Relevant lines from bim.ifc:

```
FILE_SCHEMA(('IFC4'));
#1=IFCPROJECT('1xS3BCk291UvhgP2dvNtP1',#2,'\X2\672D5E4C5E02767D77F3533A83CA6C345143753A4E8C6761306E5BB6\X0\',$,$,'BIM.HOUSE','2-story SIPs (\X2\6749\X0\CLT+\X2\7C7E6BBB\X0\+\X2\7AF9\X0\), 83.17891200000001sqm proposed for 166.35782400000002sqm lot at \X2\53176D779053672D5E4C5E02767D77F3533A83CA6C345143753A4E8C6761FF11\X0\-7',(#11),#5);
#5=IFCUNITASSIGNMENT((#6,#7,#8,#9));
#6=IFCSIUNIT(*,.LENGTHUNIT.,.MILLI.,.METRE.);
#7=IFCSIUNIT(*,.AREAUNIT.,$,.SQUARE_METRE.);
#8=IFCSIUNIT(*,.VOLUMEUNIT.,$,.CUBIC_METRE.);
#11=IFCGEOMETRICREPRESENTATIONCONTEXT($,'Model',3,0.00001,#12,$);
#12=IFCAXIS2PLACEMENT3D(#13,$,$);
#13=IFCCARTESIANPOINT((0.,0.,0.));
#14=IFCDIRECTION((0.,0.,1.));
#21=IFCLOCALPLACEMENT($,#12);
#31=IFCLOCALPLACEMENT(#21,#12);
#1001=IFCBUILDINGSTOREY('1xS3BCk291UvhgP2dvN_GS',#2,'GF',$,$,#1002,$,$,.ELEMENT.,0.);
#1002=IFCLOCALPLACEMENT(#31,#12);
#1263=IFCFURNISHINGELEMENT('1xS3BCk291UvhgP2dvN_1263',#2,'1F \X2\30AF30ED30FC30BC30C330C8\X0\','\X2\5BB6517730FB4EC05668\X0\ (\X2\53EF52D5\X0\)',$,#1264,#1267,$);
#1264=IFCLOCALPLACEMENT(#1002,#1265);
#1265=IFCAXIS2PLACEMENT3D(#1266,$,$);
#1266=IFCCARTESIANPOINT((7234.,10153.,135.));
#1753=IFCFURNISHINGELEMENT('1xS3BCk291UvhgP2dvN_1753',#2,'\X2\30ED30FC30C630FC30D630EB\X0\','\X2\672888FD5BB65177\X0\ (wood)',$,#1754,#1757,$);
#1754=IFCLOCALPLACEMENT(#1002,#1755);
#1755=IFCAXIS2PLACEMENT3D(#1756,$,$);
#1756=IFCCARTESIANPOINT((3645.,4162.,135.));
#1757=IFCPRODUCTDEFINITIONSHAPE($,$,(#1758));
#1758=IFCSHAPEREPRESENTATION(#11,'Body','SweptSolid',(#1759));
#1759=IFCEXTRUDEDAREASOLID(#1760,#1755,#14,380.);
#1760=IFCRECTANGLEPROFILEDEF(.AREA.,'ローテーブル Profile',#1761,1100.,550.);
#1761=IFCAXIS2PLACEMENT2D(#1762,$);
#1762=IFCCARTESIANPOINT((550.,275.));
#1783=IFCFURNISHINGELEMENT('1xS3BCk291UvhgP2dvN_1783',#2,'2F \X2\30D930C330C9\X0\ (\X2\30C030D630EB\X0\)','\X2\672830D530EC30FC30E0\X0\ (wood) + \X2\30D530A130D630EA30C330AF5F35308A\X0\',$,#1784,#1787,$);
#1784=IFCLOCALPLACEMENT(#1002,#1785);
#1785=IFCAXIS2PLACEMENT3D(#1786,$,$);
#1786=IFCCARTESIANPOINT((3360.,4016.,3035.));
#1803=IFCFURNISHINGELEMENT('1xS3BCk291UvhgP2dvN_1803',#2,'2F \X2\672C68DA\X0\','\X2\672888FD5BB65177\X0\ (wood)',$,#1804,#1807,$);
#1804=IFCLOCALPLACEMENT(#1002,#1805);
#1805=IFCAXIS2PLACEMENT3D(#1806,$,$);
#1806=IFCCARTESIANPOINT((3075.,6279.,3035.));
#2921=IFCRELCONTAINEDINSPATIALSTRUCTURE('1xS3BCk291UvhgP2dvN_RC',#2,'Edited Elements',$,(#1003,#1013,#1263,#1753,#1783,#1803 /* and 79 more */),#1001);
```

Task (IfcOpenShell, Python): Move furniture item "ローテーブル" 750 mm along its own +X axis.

```python
import ifcopenshell
import ifcopenshell.api.geometry
import ifcopenshell.util.placement
import ifcopenshell.util.unit

model = ifcopenshell.open("bim.ifc")
unit_scale = ifcopenshell.util.unit.calculate_unit_scale(model)

item = model.by_id(1753)
matrix = ifcopenshell.util.placement.get_local_placement(item.ObjectPlacement)
matrix[:3, 3] += matrix[:3, 0] * 0.75 / unit_scale
ifcopenshell.api.geometry.edit_object_placement(model, product=item, matrix=matrix, is_si=False)

print(ifcopenshell.util.placement.get_local_placement(item.ObjectPlacement).round(3) + 0.0)

model.write("bim_edited.ifc")
```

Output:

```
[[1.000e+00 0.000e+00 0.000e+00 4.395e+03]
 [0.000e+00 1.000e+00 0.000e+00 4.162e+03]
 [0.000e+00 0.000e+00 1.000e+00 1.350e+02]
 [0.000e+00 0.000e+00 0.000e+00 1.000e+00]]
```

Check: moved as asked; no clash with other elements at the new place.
